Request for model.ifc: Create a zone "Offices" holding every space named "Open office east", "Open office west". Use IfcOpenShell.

First a look at what the model holds.

```python
import ifcopenshell

model = ifcopenshell.open("model.ifc")
print(model.schema)
seen = {}
for space in model.by_type("IfcSpace"):
    seen[space.Name] = seen.get(space.Name, 0) + 1
for name, count in sorted(seen.items(), key=str):
    print(count, "x", name)
print("zones:", [z.Name for z in model.by_type("IfcZone")][:20])
```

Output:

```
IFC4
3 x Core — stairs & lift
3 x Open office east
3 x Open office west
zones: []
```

```python
import ifcopenshell
import ifcopenshell.api.group
import ifcopenshell.api.root

model = ifcopenshell.open("model.ifc")

names = {"Open office east", "Open office west"}
spaces = [s for s in model.by_type("IfcSpace") if s.Name in names]

zone = ifcopenshell.api.root.create_entity(model, ifc_class="IfcZone", name="Offices")
ifcopenshell.api.group.assign_group(model, products=spaces, group=zone)
print(len(spaces), "spaces in", zone.Name)

model.write("model_rev.ifc")
```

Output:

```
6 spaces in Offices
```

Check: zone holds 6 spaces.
